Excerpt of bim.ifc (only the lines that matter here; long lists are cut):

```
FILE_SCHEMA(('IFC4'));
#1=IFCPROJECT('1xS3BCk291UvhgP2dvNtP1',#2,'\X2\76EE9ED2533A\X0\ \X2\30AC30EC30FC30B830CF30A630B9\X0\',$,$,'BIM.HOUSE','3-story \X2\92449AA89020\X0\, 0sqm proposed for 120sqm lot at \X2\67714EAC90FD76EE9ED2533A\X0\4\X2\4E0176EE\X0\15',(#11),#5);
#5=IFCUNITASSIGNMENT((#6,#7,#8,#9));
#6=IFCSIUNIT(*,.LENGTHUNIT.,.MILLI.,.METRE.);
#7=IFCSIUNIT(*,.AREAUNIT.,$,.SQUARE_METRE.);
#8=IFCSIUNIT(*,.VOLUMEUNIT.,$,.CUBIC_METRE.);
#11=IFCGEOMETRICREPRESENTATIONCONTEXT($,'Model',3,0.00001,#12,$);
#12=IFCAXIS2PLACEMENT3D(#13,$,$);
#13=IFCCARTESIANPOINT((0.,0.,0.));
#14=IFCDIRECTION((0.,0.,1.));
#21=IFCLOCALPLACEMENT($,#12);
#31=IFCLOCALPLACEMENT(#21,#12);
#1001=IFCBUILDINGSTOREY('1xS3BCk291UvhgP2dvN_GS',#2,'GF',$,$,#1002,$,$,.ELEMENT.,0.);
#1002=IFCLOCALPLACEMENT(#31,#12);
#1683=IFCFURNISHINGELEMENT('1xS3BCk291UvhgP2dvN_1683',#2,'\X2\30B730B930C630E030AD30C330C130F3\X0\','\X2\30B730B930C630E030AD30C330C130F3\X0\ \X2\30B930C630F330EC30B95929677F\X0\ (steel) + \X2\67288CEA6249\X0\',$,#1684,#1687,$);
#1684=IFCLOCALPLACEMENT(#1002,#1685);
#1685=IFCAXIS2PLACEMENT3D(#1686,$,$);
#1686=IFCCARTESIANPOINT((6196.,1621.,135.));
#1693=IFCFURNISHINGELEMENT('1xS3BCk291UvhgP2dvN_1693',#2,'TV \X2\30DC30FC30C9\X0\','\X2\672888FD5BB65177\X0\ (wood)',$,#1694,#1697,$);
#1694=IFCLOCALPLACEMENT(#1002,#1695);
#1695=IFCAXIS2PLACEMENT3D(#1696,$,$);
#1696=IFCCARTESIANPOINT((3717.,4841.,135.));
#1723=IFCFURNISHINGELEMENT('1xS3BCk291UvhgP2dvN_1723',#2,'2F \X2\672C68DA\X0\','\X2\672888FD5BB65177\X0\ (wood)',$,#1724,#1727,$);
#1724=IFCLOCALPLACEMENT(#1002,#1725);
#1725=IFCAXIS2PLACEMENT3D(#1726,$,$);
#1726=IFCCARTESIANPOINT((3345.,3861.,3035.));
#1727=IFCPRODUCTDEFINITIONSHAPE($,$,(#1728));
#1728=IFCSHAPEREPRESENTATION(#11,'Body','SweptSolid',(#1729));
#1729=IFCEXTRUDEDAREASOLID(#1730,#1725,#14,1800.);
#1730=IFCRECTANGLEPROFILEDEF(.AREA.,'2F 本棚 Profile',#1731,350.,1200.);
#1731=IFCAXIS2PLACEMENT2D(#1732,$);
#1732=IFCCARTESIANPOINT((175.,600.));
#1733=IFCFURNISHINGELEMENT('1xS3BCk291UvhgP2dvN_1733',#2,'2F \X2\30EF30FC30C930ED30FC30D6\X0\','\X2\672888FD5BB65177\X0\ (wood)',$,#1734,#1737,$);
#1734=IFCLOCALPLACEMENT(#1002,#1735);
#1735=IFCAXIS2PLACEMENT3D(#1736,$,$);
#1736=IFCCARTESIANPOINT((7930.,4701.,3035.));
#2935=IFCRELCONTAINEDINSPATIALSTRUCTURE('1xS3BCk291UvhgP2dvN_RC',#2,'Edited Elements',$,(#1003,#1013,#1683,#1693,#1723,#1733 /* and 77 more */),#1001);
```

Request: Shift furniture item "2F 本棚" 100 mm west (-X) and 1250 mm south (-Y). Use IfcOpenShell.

```python
import ifcopenshell
import ifcopenshell.api.geometry
import ifcopenshell.util.placement
import ifcopenshell.util.unit

model = ifcopenshell.open("bim.ifc")
unit_scale = ifcopenshell.util.unit.calculate_unit_scale(model)

item = model.by_guid("1xS3BCk291UvhgP2dvN_1723")
matrix = ifcopenshell.util.placement.get_local_placement(item.ObjectPlacement)
matrix[0, 3] -= 0.1 / unit_scale
matrix[1, 3] -= 1.25 / unit_scale
ifcopenshell.api.geometry.edit_object_placement(model, product=item, matrix=matrix, is_si=False)

print(ifcopenshell.util.placement.get_local_placement(item.ObjectPlacement).round(3) + 0.0)

model.write("bim_edited.ifc")
```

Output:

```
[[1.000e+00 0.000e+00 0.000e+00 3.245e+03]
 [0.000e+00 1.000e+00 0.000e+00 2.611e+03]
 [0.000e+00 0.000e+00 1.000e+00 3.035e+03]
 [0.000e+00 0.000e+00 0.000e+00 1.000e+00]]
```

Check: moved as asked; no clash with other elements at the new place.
